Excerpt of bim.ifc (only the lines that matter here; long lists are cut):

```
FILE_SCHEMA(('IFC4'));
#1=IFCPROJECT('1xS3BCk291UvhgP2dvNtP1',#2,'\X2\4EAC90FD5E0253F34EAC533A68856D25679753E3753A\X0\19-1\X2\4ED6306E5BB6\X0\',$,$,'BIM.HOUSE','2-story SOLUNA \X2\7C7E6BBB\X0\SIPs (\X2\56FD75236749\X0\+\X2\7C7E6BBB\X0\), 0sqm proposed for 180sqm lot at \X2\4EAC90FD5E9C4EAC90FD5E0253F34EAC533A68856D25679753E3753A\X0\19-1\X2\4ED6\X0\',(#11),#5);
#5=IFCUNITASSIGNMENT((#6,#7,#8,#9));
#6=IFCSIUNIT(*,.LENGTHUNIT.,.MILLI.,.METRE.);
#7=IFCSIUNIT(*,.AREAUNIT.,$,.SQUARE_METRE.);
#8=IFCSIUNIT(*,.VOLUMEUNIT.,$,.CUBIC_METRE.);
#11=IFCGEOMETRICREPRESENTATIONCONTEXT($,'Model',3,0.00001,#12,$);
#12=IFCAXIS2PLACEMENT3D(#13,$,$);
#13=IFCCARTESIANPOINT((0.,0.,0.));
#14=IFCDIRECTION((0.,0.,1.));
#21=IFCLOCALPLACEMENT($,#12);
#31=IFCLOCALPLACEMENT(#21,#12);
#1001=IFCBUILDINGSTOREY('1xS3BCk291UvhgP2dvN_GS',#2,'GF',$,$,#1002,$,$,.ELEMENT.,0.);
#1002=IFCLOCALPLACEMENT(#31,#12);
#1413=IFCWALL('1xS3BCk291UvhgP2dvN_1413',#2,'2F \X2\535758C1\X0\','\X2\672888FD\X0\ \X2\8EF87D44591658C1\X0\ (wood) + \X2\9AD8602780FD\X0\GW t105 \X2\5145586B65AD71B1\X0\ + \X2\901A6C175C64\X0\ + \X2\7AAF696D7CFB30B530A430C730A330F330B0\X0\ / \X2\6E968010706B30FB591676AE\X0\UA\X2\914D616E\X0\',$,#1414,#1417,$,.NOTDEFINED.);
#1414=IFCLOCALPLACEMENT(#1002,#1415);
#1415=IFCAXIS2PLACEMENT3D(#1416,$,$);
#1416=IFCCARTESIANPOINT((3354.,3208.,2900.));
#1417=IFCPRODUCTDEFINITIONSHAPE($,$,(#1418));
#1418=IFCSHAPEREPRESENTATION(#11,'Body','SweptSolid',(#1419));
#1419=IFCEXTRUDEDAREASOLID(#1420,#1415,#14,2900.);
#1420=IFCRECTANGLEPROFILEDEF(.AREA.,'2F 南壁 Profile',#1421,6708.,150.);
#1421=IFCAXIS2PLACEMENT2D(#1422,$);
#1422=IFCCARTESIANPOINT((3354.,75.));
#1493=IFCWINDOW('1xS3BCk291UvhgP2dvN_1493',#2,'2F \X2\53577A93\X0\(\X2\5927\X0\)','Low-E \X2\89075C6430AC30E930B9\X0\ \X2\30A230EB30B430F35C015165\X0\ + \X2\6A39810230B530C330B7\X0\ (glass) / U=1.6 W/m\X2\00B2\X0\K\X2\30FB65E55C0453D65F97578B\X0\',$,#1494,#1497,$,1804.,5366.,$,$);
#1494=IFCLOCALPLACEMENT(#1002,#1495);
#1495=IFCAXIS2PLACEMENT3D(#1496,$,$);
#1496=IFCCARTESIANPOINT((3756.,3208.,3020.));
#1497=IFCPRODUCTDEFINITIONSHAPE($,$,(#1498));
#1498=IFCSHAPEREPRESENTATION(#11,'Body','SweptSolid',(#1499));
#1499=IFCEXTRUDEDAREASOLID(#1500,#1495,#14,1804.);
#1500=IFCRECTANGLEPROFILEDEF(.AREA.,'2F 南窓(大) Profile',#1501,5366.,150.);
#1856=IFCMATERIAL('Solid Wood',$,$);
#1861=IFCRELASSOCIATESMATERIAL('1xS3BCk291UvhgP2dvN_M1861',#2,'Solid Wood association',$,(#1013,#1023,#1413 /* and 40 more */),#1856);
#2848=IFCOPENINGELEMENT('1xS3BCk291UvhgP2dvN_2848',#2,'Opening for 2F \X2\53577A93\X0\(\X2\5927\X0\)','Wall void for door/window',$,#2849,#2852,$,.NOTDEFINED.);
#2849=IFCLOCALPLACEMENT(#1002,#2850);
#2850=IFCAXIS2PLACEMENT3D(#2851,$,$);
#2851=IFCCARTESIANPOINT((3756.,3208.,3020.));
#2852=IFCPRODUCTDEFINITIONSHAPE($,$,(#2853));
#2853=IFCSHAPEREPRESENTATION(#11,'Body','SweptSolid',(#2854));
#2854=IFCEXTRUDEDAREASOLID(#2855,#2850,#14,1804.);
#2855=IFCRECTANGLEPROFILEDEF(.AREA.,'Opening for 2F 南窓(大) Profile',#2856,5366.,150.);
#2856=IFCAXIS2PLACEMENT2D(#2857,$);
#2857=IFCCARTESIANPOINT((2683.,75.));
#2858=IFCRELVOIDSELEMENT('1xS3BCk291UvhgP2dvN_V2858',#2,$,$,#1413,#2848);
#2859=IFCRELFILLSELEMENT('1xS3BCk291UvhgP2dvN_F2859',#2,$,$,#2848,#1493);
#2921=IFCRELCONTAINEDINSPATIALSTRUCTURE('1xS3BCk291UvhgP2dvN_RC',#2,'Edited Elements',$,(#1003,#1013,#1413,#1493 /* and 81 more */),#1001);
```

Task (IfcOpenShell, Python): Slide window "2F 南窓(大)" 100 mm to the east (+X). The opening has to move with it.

```python
import ifcopenshell
import ifcopenshell.api.geometry
import ifcopenshell.util.placement
import ifcopenshell.util.unit

model = ifcopenshell.open("bim.ifc")
unit_scale = ifcopenshell.util.unit.calculate_unit_scale(model)

window = model.by_guid("1xS3BCk291UvhgP2dvN_1493")
opening = window.FillsVoids[0].RelatingOpeningElement
wall = opening.VoidsElements[0].RelatingBuildingElement

wall_matrix = ifcopenshell.util.placement.get_local_placement(wall.ObjectPlacement)
shift = wall_matrix[:3, 0] * 0.1 / unit_scale
before = ifcopenshell.util.placement.get_local_placement(window.ObjectPlacement)[:3, 3].copy()

# The window is not placed relative to its opening, so move both.
for product in (opening, window):
    matrix = ifcopenshell.util.placement.get_local_placement(product.ObjectPlacement)
    matrix[:3, 3] += shift
    ifcopenshell.api.geometry.edit_object_placement(model, product=product, matrix=matrix, is_si=False)

after = ifcopenshell.util.placement.get_local_placement(window.ObjectPlacement)[:3, 3]
print("window moved by", (after - before).round(3) + 0.0)

model.write("bim_v2.ifc")
```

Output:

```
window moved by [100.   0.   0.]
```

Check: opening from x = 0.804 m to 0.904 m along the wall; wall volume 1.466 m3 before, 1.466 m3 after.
